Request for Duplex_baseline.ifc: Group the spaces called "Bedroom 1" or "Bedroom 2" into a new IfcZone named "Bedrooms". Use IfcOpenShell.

First a look at what the model holds.

```python
import ifcopenshell

model = ifcopenshell.open("Duplex_baseline.ifc")
print(model.schema)
seen = {}
for space in model.by_type("IfcSpace"):
    seen[space.LongName] = seen.get(space.LongName, 0) + 1
for name, count in sorted(seen.items(), key=str):
    print(count, "x", name)
print("zones:", [z.Name for z in model.by_type("IfcZone")][:20])
```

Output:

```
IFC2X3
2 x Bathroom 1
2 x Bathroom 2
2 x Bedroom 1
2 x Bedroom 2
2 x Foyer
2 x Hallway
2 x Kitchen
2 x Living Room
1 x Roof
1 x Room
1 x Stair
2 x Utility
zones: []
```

```python
import ifcopenshell
import ifcopenshell.api.group
import ifcopenshell.api.root

model = ifcopenshell.open("Duplex_baseline.ifc")

names = {"Bedroom 1", "Bedroom 2"}
spaces = [s for s in model.by_type("IfcSpace") if s.LongName in names]

zone = ifcopenshell.api.root.create_entity(model, ifc_class="IfcZone", name="Bedrooms")
ifcopenshell.api.group.assign_group(model, products=spaces, group=zone)
print(len(spaces), "spaces in", zone.Name)

model.write("Duplex_baseline_edited.ifc")
```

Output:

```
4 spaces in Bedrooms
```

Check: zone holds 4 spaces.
